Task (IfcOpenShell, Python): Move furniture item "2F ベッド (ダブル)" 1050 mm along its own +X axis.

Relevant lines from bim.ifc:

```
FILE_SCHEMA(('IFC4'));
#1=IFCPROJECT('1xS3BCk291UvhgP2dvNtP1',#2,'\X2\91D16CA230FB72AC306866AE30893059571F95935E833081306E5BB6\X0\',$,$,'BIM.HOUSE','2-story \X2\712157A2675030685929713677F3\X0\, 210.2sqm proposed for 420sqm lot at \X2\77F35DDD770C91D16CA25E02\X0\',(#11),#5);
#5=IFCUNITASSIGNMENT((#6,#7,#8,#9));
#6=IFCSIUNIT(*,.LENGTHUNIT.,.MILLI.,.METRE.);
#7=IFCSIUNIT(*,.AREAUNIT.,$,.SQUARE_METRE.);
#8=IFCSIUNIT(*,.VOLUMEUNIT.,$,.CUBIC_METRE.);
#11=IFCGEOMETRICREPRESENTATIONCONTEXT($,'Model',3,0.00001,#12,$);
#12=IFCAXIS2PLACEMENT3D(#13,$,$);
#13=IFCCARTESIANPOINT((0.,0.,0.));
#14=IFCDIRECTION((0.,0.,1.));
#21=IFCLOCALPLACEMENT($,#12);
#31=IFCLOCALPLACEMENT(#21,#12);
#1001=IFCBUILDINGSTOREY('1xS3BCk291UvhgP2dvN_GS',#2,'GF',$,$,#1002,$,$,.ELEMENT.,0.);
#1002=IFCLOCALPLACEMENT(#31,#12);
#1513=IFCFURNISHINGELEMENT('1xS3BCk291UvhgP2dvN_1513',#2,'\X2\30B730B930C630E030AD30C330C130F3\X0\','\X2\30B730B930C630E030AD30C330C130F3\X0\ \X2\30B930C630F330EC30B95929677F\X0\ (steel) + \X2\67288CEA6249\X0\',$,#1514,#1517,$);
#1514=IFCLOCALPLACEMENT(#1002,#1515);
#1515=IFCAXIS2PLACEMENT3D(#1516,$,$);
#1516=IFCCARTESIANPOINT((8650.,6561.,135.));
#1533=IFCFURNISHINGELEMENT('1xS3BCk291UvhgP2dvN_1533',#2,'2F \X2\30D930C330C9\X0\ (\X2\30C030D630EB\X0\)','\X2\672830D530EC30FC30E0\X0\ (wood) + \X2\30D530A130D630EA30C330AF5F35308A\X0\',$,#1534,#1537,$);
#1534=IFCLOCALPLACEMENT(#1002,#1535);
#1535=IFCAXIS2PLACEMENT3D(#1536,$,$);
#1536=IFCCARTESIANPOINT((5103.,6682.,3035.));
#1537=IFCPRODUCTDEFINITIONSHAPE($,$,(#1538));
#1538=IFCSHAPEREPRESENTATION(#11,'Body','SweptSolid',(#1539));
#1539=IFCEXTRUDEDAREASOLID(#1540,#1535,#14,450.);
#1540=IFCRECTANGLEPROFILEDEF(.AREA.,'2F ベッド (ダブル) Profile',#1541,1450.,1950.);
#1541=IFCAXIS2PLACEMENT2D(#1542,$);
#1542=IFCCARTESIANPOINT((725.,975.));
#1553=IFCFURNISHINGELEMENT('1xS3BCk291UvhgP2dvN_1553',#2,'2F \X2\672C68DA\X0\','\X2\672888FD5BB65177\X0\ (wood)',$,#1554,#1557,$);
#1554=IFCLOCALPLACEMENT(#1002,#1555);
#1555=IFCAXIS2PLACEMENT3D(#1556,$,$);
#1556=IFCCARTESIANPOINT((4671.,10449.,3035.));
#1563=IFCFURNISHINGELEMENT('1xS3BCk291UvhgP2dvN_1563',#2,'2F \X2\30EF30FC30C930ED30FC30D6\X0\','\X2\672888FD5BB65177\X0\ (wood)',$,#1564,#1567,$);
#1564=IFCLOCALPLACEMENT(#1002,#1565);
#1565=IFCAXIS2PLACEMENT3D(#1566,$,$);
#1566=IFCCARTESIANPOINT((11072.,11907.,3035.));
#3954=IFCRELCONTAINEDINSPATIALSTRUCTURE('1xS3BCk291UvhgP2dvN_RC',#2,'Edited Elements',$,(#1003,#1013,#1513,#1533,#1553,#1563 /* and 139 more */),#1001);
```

```python
import ifcopenshell
import ifcopenshell.api.geometry
import ifcopenshell.util.placement

model = ifcopenshell.open("bim.ifc")

item = model.by_guid("1xS3BCk291UvhgP2dvN_1533")
matrix = ifcopenshell.util.placement.get_local_placement(item.ObjectPlacement)
matrix[:3, 3] += matrix[:3, 0] * 1050.0
ifcopenshell.api.geometry.edit_object_placement(model, product=item, matrix=matrix, is_si=False)

print(ifcopenshell.util.placement.get_local_placement(item.ObjectPlacement).round(3) + 0.0)

model.write("bim_v2.ifc")
```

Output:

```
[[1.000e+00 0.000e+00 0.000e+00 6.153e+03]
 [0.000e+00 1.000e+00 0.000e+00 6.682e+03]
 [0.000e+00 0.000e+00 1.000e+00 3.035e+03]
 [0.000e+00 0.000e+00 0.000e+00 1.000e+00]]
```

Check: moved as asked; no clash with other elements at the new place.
